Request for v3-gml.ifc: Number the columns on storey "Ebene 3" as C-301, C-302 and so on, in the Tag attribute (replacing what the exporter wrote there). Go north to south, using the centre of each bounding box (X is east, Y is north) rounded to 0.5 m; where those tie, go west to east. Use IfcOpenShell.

First a look at what the model holds.

```python
import ifcopenshell
import ifcopenshell.util.element
import ifcopenshell.util.placement

model = ifcopenshell.open("v3-gml.ifc")
print(model.schema)
storey = next(s for s in model.by_type("IfcBuildingStorey") if s.Name == "Ebene 3")
columns = [e for e in ifcopenshell.util.element.get_decomposition(storey) if e.is_a("IfcColumn")]
for e in sorted(columns, key=lambda e: e.id()):
    origin = ifcopenshell.util.placement.get_local_placement(e.ObjectPlacement)[:3, 3]
    print(e.id(), e.Tag, e.Name, origin.round(2) + 0.0, sep=" | ")
```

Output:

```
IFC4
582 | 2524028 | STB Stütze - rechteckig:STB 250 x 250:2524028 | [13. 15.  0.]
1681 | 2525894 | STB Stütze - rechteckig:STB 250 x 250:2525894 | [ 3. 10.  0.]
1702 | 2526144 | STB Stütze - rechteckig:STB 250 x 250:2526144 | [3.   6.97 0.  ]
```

```python
import ifcopenshell
import ifcopenshell.geom
import ifcopenshell.util.element
import ifcopenshell.util.shape

model = ifcopenshell.open("v3-gml.ifc")
settings = ifcopenshell.geom.settings()
settings.set("use-world-coords", True)


def centre(element):
    shape = ifcopenshell.geom.create_shape(settings, element)
    return ifcopenshell.util.shape.get_bbox_centroid(shape.geometry)


storey = next(s for s in model.by_type("IfcBuildingStorey") if s.Name == "Ebene 3")
columns = [e for e in ifcopenshell.util.element.get_decomposition(storey) if e.is_a("IfcColumn")]

# Insertion points can sit at a corner or the storey origin, so sort by the geometry (in metres).
centres = {e: centre(e) for e in columns}
columns.sort(key=lambda e: (-round(centres[e][1] / 0.5), centres[e][0]))

for i, e in enumerate(columns, start=1):
    number = f"C-3{i:02d}"
    e.Tag = number
    print(e.id(), number)

model.write("v3-gml_updated.ifc")
```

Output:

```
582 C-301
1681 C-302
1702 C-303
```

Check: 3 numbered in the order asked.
